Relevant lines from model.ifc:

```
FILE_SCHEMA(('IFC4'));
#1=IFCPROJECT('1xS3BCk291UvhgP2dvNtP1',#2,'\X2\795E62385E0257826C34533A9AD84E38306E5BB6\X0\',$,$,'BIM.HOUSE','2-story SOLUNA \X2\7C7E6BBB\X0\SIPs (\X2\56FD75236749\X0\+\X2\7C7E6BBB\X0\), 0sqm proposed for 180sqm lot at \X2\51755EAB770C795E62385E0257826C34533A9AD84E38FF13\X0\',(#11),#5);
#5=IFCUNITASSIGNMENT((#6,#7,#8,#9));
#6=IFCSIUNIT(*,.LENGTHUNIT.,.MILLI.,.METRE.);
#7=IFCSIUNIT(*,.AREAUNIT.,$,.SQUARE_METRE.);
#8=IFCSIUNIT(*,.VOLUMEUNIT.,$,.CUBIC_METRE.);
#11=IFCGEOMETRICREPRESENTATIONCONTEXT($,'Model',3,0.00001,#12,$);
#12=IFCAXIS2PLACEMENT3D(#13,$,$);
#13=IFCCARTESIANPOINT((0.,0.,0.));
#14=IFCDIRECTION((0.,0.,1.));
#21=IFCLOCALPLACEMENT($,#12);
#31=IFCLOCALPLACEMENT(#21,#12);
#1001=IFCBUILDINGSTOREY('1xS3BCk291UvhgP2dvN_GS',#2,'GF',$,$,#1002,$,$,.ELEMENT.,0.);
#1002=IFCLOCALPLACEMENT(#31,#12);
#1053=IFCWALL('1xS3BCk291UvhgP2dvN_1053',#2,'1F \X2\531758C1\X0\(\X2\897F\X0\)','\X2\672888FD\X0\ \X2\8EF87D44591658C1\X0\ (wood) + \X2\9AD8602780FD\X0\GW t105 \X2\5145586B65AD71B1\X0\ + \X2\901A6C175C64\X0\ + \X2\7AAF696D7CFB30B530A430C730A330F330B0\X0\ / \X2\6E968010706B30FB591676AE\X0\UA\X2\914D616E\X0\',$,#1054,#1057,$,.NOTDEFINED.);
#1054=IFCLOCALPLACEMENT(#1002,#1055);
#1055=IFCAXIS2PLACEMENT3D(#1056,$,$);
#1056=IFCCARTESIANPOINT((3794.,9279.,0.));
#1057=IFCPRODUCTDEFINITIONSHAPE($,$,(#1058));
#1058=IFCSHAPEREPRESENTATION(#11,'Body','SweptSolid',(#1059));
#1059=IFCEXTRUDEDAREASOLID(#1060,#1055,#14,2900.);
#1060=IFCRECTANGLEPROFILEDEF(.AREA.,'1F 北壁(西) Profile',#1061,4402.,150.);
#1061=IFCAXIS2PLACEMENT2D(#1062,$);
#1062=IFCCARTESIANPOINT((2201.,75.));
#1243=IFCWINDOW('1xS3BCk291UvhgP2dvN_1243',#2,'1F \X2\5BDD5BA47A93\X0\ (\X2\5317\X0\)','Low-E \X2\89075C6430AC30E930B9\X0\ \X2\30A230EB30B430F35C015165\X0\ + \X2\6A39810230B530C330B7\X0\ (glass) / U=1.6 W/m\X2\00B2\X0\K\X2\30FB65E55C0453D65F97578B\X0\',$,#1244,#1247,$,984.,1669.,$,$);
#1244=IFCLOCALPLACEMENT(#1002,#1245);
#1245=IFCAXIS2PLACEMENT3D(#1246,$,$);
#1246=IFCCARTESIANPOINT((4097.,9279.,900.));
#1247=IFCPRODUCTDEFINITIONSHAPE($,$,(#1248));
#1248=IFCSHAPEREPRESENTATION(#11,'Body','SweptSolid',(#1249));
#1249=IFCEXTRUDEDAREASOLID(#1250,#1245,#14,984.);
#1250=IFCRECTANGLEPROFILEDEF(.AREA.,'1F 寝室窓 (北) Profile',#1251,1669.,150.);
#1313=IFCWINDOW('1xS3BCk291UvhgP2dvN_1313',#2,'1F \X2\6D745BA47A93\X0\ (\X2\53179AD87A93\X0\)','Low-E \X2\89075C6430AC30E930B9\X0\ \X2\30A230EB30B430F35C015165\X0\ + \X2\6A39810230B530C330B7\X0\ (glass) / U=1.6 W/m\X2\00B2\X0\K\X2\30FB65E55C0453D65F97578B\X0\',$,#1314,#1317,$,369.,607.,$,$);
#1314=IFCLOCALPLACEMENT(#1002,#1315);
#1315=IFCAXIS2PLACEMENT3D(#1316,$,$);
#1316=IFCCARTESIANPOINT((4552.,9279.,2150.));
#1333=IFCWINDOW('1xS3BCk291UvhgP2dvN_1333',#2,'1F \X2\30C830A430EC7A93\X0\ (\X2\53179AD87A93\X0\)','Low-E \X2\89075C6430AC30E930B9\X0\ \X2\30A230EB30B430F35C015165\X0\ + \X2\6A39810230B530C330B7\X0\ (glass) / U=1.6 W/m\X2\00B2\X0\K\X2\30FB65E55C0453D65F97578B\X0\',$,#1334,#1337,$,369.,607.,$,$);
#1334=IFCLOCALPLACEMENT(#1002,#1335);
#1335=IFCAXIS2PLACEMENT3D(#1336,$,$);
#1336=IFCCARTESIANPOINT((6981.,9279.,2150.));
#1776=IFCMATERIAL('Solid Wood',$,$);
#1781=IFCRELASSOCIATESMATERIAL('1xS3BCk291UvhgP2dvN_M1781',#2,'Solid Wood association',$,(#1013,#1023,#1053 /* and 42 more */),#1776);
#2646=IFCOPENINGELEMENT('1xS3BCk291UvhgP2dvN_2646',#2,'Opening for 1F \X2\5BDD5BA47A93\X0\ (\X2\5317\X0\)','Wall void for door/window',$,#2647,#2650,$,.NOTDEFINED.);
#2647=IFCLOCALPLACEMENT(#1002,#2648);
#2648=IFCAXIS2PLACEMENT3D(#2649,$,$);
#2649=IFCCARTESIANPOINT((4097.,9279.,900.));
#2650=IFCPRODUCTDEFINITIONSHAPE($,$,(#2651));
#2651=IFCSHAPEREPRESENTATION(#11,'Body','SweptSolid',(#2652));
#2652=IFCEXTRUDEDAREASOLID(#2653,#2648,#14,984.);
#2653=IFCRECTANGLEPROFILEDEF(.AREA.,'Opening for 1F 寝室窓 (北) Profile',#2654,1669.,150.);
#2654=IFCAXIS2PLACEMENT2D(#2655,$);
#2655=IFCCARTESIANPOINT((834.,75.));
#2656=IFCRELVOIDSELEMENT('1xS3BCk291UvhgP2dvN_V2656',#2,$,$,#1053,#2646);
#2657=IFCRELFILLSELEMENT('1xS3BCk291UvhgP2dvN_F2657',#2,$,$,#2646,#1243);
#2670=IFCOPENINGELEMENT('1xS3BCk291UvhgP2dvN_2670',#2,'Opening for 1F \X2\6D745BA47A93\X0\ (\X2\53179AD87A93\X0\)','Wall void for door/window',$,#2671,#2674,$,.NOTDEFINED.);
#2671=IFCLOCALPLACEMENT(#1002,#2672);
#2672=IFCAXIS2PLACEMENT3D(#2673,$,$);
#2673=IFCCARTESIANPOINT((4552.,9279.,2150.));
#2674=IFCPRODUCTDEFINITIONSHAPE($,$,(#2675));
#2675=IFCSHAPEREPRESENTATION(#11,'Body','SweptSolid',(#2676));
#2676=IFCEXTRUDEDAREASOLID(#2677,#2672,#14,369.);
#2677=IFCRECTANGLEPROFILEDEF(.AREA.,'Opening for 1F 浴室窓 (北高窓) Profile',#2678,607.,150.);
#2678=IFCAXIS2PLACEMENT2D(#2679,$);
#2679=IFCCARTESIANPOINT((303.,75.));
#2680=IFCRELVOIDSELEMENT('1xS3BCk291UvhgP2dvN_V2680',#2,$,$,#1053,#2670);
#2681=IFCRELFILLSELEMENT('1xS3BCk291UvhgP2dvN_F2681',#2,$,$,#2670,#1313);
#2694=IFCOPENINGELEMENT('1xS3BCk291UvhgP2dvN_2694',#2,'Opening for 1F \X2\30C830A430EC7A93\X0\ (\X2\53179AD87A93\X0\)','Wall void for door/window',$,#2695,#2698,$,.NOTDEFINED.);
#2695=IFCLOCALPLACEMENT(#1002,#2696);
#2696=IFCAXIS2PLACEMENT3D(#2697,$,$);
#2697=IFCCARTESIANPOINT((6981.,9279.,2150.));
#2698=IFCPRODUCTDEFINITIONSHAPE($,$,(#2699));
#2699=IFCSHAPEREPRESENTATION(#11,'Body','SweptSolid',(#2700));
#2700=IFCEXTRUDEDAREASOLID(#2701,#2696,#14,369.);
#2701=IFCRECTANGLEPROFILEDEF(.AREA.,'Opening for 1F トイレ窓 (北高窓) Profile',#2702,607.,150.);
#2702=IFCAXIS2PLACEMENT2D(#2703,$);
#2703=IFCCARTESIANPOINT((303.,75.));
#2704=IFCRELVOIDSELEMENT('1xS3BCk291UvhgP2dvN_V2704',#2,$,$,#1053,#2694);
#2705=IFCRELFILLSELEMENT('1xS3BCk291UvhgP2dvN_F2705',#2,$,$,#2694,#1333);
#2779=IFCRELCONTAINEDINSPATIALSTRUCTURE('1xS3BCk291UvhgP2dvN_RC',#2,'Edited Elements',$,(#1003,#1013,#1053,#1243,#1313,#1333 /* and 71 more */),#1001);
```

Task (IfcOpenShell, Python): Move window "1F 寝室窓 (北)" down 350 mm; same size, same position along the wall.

```python
import numpy as np
import ifcopenshell
import ifcopenshell.api.geometry
import ifcopenshell.util.placement
import ifcopenshell.util.unit

model = ifcopenshell.open("model.ifc")
unit_scale = ifcopenshell.util.unit.calculate_unit_scale(model)

window = model.by_guid("1xS3BCk291UvhgP2dvN_1243")
opening = window.FillsVoids[0].RelatingOpeningElement
dz = -350.0

shift = np.array([0.0, 0.0, dz])
# The window is not placed relative to its opening, so move both.
for product in (opening, window):
    matrix = ifcopenshell.util.placement.get_local_placement(product.ObjectPlacement)
    matrix[:3, 3] += shift
    ifcopenshell.api.geometry.edit_object_placement(model, product=product, matrix=matrix, is_si=False)

print(f"moved by {dz * unit_scale:+.3f} m")

model.write("model_v2.ifc")
```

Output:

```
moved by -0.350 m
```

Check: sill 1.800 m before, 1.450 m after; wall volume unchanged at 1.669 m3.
